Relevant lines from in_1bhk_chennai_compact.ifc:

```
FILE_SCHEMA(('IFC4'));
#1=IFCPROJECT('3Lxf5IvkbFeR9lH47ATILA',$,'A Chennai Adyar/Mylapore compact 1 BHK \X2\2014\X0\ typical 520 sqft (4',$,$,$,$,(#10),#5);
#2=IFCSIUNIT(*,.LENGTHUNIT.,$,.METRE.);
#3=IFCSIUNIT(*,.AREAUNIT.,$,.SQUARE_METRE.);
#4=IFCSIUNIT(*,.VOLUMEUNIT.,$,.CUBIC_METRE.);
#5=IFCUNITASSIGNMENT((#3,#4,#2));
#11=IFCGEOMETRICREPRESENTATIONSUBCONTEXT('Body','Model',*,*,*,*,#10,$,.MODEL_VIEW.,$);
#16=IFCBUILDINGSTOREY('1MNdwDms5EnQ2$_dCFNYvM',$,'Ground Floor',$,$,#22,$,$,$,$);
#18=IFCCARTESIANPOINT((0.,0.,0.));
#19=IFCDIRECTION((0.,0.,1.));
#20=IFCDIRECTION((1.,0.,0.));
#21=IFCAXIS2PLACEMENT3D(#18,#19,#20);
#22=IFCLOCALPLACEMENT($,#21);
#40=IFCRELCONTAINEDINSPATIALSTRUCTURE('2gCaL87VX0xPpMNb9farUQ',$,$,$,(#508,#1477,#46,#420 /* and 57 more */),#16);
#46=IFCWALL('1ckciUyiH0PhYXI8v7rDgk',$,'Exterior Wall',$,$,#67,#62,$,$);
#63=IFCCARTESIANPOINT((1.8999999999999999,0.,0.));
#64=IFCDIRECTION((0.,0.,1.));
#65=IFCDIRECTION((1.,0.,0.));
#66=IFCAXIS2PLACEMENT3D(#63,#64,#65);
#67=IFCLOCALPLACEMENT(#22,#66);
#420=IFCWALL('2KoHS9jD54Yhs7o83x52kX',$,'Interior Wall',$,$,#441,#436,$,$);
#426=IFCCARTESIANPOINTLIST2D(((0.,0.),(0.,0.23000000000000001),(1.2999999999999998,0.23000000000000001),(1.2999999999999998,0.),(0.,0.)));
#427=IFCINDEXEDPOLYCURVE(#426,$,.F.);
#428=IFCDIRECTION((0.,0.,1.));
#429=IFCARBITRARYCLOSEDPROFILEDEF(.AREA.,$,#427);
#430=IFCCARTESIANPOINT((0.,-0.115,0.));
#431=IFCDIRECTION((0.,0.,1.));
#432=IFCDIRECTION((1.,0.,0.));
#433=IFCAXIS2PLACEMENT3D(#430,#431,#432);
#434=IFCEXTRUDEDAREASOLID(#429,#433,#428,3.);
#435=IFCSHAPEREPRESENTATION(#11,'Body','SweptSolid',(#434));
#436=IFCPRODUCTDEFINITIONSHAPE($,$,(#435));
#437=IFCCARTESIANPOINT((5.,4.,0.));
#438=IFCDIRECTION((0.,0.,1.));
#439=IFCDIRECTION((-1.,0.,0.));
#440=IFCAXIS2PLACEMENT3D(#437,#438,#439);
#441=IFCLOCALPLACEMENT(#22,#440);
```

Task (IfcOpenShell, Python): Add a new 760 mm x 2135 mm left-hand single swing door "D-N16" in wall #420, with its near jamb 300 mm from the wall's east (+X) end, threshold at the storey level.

```python
import numpy as np
import ifcopenshell
import ifcopenshell.api.feature
import ifcopenshell.api.geometry
import ifcopenshell.api.root
import ifcopenshell.api.spatial
import ifcopenshell.geom
import ifcopenshell.util.element
import ifcopenshell.util.placement
import ifcopenshell.util.representation
import ifcopenshell.util.shape
import ifcopenshell.util.unit

model = ifcopenshell.open("in_1bhk_chennai_compact.ifc")
unit_scale = ifcopenshell.util.unit.calculate_unit_scale(model)
settings = ifcopenshell.geom.settings()


def volume(element):
    """Net volume in cubic metres, openings subtracted."""
    shape = ifcopenshell.geom.create_shape(settings, element)
    return ifcopenshell.util.shape.get_volume(shape.geometry)


wall = model.by_guid("2KoHS9jD54Yhs7o83x52kX")
storey = ifcopenshell.util.element.get_container(wall, ifc_class="IfcBuildingStorey")
context = ifcopenshell.util.representation.get_context(model, "Model", "Body", "MODEL_VIEW")
before = volume(wall)

width, height, from_end, sill = 0.76, 2.135, 0.3, 0.0  # metres

# The wall runs along its own X axis, and the end named is its -X end.
wall_shape = ifcopenshell.geom.create_shape(settings, wall)
x, y, z = ifcopenshell.util.shape.get_vertices(wall_shape.geometry).T
start = x.min() + from_end
face, thickness = float(y.min()), float(y.max() - y.min())
wall_matrix = ifcopenshell.util.placement.get_local_placement(wall.ObjectPlacement)
level = ifcopenshell.util.placement.get_local_placement(storey.ObjectPlacement)[2, 3]


def in_wall(x, y):
    """Placement at x, y metres in the wall's axes, at sill height."""
    matrix = wall_matrix.copy()
    matrix[:, 3] = wall_matrix @ np.array([x / unit_scale, y / unit_scale, 0.0, 1.0])
    matrix[2, 3] = level + sill / unit_scale
    return matrix


# Opening: a box that overshoots both wall faces by 50 mm.
opening = ifcopenshell.api.root.create_entity(model, ifc_class="IfcOpeningElement", predefined_type="OPENING")
box = ifcopenshell.api.geometry.add_wall_representation(
    model, context=context, length=width, height=height, thickness=thickness + 0.1
)
ifcopenshell.api.geometry.assign_representation(model, product=opening, representation=box)
ifcopenshell.api.geometry.edit_object_placement(model, product=opening, matrix=in_wall(start, face - 0.05), is_si=False)
ifcopenshell.api.feature.add_feature(model, feature=opening, element=wall)

door = ifcopenshell.api.root.create_entity(model, ifc_class="IfcDoor", name="D-N16", predefined_type="DOOR")
door.OverallWidth, door.OverallHeight = width / unit_scale, height / unit_scale
door.OperationType = "SINGLE_SWING_LEFT"
body = ifcopenshell.api.geometry.add_door_representation(
    model,
    context=context,
    overall_width=door.OverallWidth,
    overall_height=door.OverallHeight,
    operation_type="SINGLE_SWING_LEFT",
    lining_properties={"LiningDepth": thickness / unit_scale, "ThresholdDepth": thickness / unit_scale},
)
ifcopenshell.api.geometry.assign_representation(model, product=door, representation=body)
ifcopenshell.api.spatial.assign_container(model, products=[door], relating_structure=storey)
ifcopenshell.api.feature.add_filling(model, opening=opening, element=door)

# The lining spans the wall, so the door starts at the wall face.
ifcopenshell.api.geometry.edit_object_placement(model, product=door, matrix=in_wall(start, face), is_si=False)

after = volume(wall)

print(f"wall volume {before:.3f} -> {after:.3f} m3")

model.write("in_1bhk_chennai_compact_updated.ifc")
```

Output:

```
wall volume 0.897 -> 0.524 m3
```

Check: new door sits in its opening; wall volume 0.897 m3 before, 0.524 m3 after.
